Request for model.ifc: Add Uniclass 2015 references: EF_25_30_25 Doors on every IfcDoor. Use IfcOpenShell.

First a look at what the model holds.

```python
import ifcopenshell

model = ifcopenshell.open("model.ifc")
print(model.schema)
print("classifications:", [c.Name for c in model.by_type("IfcClassification")])
for ifc_class in ("IfcDoor", "IfcRoof", "IfcStair", "IfcWall", "IfcWindow"):
    print(ifc_class, len(model.by_type(ifc_class)))
```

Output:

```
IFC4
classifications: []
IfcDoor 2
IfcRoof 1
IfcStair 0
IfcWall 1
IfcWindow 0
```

```python
import ifcopenshell
import ifcopenshell.api.classification

model = ifcopenshell.open("model.ifc")

system = ifcopenshell.api.classification.add_classification(model, classification="Uniclass 2015")

codes = {
    "IfcDoor": ("EF_25_30_25", "Doors"),
}
for ifc_class, (code, name) in codes.items():
    products = model.by_type(ifc_class)
    ifcopenshell.api.classification.add_reference(
        model, products=products, classification=system, identification=code, name=name
    )
    print(code, len(products))

model.write("model-out.ifc")
```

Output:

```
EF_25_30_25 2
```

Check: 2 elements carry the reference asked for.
